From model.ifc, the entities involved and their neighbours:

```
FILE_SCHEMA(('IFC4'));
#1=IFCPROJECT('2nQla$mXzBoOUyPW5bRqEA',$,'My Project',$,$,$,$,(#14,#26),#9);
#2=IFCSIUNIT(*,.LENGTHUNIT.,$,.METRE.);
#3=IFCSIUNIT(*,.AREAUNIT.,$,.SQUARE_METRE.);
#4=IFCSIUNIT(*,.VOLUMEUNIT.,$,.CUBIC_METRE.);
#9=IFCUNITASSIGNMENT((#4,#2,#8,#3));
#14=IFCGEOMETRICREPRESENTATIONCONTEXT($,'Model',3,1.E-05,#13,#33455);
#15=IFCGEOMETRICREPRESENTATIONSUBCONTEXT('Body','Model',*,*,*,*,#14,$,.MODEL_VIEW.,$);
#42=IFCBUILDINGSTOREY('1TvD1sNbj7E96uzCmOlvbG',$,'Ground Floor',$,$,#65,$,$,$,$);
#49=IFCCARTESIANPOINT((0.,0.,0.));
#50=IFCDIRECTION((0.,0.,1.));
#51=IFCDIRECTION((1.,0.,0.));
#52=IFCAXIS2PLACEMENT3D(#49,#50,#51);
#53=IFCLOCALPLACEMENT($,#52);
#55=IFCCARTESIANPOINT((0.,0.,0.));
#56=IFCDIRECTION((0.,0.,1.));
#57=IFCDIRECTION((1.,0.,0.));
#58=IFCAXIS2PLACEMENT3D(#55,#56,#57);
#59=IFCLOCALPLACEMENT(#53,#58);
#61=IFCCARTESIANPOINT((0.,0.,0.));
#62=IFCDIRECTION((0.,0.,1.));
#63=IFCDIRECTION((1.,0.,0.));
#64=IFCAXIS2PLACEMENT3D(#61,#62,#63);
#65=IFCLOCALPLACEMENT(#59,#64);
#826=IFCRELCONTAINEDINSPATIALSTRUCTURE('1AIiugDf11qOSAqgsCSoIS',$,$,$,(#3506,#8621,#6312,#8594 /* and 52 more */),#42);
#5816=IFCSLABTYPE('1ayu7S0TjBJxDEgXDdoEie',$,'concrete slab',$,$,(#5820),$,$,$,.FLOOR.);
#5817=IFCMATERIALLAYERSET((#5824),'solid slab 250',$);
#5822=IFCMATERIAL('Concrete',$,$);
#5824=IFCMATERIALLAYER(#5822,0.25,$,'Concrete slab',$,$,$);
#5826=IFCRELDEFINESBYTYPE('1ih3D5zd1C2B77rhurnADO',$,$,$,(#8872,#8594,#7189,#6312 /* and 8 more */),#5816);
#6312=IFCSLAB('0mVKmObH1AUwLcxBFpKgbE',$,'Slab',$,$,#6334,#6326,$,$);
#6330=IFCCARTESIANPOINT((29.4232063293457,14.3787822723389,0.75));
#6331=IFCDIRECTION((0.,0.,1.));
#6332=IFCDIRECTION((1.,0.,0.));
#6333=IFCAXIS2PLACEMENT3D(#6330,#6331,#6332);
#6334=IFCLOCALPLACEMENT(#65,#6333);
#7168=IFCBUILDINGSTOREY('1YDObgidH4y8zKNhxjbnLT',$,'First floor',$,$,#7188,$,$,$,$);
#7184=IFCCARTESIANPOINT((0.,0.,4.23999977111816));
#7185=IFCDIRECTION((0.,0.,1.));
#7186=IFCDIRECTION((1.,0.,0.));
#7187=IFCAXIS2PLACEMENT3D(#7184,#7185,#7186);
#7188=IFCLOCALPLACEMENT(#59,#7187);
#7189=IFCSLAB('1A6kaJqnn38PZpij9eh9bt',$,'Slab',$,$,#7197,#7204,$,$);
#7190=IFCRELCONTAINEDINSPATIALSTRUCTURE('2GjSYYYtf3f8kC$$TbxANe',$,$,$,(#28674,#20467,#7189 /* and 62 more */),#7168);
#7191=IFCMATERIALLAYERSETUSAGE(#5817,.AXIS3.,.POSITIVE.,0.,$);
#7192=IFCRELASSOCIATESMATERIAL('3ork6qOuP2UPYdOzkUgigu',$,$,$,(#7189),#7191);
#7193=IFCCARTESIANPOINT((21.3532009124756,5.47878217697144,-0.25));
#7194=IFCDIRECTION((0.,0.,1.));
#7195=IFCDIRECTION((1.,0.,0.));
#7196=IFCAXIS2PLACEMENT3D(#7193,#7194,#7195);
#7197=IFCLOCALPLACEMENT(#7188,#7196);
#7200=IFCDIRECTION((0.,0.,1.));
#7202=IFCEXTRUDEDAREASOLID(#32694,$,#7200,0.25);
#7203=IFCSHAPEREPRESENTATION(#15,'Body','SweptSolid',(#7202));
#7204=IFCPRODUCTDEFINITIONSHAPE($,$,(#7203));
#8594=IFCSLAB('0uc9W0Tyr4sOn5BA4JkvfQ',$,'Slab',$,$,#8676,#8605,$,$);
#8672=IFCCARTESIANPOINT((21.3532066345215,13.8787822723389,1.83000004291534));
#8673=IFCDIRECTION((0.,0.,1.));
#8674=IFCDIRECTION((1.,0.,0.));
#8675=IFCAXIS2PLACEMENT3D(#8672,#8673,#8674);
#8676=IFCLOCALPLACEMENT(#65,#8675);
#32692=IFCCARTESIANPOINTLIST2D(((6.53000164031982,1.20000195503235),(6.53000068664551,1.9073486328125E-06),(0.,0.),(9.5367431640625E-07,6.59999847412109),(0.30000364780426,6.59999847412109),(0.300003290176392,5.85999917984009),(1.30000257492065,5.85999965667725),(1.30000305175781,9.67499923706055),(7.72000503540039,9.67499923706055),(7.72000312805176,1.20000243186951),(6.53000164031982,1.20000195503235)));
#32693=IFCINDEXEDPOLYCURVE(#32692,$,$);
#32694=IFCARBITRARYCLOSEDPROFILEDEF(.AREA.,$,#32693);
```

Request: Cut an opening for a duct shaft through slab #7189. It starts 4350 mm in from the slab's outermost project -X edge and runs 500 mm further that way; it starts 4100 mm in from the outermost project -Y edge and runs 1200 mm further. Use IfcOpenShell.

```python
import numpy as np
import ifcopenshell
import ifcopenshell.api.feature
import ifcopenshell.api.geometry
import ifcopenshell.api.root
import ifcopenshell.geom
import ifcopenshell.util.placement
import ifcopenshell.util.representation
import ifcopenshell.util.shape
import ifcopenshell.util.unit

model = ifcopenshell.open("model.ifc")
unit_scale = ifcopenshell.util.unit.calculate_unit_scale(model)
settings = ifcopenshell.geom.settings()


def volume(element):
    """Net volume in cubic metres, openings subtracted."""
    shape = ifcopenshell.geom.create_shape(settings, element)
    return ifcopenshell.util.shape.get_volume(shape.geometry)


slab = model.by_guid("1A6kaJqnn38PZpij9eh9bt")
before = volume(slab)

# Extent in the slab's own axes, in metres. The edges named are its -X and -Y sides.
slab_shape = ifcopenshell.geom.create_shape(settings, slab)
vertices = ifcopenshell.util.shape.get_vertices(slab_shape.geometry)
x_min, y_min, bottom = vertices.min(axis=0)
top = vertices[:, 2].max()

opening = ifcopenshell.api.root.create_entity(model, ifc_class="IfcOpeningElement", name="Duct shaft opening", predefined_type="OPENING")
context = ifcopenshell.util.representation.get_context(model, "Model", "Body", "MODEL_VIEW")
width, depth = 0.5, 1.2
outline = [(0.0, 0.0), (width, 0.0), (width, depth), (0.0, depth), (0.0, 0.0)]
# Overshoot both faces by 50 mm so the cut is clean.
shape = ifcopenshell.api.geometry.add_slab_representation(
    model, context=context, depth=top - bottom + 0.1, polyline=outline
)
ifcopenshell.api.geometry.assign_representation(model, product=opening, representation=shape)

matrix = ifcopenshell.util.placement.get_local_placement(slab.ObjectPlacement)
matrix[:, 3] = matrix @ np.append(np.array([x_min + 4.35, y_min + 4.1, bottom - 0.05]) / unit_scale, 1.0)
ifcopenshell.api.geometry.edit_object_placement(model, product=opening, matrix=matrix, is_si=False)
ifcopenshell.api.feature.add_feature(model, feature=opening, element=slab)

after = volume(slab)

print(f"slab volume {before:.3f} -> {after:.3f} m3")

model.write("model_edited.ifc")
```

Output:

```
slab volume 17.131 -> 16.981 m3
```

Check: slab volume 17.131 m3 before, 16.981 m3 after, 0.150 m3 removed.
